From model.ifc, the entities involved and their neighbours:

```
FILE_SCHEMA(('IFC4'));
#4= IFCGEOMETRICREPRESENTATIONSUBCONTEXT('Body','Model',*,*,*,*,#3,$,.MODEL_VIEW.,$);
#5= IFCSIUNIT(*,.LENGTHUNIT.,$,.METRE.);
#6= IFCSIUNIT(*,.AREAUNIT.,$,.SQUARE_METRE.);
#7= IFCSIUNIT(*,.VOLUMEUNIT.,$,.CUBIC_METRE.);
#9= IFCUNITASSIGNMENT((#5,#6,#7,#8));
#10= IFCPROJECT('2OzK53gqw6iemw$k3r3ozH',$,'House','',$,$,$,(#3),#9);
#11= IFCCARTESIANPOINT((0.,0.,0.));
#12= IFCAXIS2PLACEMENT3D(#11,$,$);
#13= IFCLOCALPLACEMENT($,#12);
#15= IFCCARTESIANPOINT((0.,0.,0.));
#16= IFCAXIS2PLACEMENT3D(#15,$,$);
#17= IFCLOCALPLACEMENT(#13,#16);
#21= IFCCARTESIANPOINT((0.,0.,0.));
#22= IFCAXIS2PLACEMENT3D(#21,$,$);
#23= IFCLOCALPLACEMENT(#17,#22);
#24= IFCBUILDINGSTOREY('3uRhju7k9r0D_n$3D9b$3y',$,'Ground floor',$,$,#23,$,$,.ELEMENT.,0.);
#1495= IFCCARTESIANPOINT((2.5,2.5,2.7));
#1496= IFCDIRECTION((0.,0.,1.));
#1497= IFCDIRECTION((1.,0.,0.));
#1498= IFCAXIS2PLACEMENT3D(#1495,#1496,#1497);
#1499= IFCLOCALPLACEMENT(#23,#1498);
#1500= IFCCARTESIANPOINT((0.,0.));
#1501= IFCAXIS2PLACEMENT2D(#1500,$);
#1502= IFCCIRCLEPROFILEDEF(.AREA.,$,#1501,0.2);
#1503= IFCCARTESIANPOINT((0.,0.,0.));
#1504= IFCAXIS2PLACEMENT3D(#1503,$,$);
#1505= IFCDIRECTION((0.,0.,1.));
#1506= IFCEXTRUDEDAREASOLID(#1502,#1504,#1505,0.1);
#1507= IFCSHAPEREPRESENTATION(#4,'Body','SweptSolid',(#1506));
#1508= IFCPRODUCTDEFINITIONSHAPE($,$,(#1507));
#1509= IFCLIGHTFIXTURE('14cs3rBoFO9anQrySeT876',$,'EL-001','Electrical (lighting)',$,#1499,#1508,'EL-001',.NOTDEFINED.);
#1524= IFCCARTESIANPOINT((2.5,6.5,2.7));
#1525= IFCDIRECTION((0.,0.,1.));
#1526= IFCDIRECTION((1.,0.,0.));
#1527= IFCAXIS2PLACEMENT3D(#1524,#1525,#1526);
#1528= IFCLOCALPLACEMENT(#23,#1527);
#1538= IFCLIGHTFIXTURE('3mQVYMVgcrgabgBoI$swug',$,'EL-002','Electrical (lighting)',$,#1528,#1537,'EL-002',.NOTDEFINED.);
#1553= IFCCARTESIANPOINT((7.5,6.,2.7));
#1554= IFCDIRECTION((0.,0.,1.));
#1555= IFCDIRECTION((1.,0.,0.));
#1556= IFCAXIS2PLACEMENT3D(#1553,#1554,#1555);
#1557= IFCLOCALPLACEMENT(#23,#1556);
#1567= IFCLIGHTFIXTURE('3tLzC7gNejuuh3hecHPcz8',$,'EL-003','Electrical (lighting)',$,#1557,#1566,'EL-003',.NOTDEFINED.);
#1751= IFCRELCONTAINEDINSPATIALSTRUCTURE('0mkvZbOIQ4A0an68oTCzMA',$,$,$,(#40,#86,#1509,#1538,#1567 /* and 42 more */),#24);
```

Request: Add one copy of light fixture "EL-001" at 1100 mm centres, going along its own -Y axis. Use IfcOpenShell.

```python
import ifcopenshell
import ifcopenshell.api.geometry
import ifcopenshell.api.root
import ifcopenshell.util.element
import ifcopenshell.util.placement
import ifcopenshell.util.unit

model = ifcopenshell.open("model.ifc")
unit_scale = ifcopenshell.util.unit.calculate_unit_scale(model)

source = model.by_guid("14cs3rBoFO9anQrySeT876")
base = ifcopenshell.util.placement.get_local_placement(source.ObjectPlacement)
step = -base[:3, 1] * 1.1 / unit_scale

for i in range(1, 2):
    copy = ifcopenshell.api.root.copy_class(model, product=source)
    copy.Representation = ifcopenshell.util.element.copy_deep(
        model, source.Representation, exclude=["IfcGeometricRepresentationContext", "IfcRepresentationMap"]
    )
    copy.Tag = None
    matrix = base.copy()
    matrix[:3, 3] += i * step
    print("added at", matrix[:3, 3].round(3) + 0.0)
    ifcopenshell.api.geometry.edit_object_placement(model, product=copy, matrix=matrix, is_si=False)

model.write("model_v2.ifc")
```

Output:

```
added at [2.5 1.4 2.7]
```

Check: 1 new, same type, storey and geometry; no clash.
